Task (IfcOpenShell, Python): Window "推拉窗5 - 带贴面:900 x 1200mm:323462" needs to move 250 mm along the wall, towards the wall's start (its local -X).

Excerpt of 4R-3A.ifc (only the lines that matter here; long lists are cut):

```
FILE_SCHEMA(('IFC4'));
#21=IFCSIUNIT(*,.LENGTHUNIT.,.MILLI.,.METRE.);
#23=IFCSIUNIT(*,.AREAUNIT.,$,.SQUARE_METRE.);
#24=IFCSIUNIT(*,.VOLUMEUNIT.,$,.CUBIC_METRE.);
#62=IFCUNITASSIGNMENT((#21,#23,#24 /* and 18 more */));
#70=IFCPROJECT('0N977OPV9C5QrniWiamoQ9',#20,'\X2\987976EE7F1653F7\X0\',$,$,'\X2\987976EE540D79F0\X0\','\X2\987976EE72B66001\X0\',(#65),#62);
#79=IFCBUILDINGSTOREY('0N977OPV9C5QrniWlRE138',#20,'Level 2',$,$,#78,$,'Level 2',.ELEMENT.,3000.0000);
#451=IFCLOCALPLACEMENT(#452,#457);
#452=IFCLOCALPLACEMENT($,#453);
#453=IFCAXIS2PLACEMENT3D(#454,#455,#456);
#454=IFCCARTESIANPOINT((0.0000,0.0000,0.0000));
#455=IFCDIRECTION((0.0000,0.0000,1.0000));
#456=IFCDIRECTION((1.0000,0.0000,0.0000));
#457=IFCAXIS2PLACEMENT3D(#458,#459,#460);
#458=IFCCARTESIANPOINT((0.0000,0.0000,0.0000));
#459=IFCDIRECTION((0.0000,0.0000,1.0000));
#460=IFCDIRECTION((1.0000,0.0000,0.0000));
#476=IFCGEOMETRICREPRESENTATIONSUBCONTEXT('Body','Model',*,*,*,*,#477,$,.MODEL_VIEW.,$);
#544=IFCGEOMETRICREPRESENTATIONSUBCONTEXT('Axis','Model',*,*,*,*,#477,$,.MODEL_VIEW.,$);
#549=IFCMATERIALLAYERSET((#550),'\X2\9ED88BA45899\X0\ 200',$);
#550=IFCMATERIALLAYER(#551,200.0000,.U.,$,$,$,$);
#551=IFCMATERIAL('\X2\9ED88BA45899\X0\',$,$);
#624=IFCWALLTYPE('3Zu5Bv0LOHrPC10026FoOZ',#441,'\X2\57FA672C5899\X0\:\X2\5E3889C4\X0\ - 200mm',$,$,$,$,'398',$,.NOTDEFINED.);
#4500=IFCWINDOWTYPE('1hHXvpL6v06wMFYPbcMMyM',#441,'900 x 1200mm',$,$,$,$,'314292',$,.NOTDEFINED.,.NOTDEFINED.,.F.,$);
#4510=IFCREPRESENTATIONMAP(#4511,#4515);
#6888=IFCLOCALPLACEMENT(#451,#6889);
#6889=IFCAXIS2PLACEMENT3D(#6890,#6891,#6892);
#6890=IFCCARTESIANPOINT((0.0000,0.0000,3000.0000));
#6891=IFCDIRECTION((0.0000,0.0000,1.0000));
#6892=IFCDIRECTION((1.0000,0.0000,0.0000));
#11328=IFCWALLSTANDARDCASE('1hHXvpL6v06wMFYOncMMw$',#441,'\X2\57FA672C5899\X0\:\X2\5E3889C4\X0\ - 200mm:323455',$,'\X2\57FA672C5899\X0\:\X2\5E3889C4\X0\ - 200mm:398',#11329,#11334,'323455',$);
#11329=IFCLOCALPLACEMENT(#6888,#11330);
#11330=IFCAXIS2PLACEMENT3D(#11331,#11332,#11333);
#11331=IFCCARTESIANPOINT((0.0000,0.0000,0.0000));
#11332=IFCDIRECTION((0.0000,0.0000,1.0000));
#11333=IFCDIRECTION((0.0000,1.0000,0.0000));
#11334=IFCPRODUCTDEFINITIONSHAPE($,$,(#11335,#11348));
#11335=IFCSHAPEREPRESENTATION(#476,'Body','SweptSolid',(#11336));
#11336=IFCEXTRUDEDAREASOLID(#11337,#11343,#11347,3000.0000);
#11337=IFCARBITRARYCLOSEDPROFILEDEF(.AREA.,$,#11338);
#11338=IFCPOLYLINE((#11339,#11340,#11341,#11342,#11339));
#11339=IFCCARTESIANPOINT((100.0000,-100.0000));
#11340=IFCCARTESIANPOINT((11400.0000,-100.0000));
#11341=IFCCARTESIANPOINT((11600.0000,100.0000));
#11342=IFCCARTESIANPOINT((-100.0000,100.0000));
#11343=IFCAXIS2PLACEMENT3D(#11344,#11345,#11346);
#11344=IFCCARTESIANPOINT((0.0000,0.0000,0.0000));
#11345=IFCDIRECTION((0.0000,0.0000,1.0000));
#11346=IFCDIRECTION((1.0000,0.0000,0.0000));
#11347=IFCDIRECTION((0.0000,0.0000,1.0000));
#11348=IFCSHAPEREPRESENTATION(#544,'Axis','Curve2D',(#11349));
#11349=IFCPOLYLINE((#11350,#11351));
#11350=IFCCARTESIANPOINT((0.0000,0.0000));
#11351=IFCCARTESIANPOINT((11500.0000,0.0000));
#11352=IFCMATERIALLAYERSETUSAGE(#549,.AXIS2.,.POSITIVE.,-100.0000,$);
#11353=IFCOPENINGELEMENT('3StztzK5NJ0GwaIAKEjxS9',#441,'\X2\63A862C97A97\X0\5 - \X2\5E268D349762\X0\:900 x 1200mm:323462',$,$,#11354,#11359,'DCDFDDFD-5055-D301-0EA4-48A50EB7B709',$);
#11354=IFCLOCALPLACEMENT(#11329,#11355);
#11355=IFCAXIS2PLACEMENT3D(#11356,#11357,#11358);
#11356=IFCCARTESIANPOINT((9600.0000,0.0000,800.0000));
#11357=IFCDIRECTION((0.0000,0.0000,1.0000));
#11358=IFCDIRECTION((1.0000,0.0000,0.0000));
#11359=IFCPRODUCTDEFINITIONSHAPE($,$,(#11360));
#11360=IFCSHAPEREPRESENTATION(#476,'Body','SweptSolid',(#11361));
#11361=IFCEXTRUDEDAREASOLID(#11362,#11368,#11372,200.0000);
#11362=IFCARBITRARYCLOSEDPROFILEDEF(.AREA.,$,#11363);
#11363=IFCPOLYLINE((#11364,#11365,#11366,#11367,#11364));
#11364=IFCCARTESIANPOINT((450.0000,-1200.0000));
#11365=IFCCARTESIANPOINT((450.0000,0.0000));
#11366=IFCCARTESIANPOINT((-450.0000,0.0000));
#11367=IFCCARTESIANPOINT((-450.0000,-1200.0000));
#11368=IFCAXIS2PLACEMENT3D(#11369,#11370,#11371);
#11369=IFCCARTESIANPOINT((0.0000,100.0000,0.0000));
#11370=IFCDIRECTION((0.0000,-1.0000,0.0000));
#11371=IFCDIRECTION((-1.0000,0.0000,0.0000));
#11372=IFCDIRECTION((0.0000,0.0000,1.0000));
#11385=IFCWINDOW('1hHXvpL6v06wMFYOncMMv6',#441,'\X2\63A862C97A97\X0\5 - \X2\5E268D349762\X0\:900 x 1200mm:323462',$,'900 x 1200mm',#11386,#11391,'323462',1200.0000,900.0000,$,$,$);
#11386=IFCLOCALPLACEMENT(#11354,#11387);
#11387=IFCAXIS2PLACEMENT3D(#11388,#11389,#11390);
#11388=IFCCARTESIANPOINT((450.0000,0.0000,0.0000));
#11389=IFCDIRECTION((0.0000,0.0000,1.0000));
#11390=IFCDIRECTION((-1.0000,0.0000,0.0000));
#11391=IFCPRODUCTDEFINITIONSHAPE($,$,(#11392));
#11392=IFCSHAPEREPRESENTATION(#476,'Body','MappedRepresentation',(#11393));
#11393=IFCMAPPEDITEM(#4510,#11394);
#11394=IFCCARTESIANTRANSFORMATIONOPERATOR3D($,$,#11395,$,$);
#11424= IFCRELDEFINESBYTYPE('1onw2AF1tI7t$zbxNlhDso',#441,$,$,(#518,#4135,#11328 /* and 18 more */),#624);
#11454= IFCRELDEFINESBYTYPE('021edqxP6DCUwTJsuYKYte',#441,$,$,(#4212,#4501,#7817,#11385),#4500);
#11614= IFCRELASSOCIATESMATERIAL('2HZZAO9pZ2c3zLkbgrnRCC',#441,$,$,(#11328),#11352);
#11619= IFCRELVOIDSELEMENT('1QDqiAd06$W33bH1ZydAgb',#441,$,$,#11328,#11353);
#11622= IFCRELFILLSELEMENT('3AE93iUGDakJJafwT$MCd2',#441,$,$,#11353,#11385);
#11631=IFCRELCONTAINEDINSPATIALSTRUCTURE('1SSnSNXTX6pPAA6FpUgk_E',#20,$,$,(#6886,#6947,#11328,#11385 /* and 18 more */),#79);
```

```python
import ifcopenshell
import ifcopenshell.api.geometry
import ifcopenshell.util.placement
import ifcopenshell.util.unit

model = ifcopenshell.open("4R-3A.ifc")
unit_scale = ifcopenshell.util.unit.calculate_unit_scale(model)

window = model.by_guid("1hHXvpL6v06wMFYOncMMv6")
opening = window.FillsVoids[0].RelatingOpeningElement
wall = opening.VoidsElements[0].RelatingBuildingElement

wall_matrix = ifcopenshell.util.placement.get_local_placement(wall.ObjectPlacement)
shift = wall_matrix[:3, 0] * -0.25 / unit_scale
before = ifcopenshell.util.placement.get_local_placement(window.ObjectPlacement)[:3, 3].copy()

# The window is placed relative to its opening, so it follows when the opening moves.
matrix = ifcopenshell.util.placement.get_local_placement(opening.ObjectPlacement)
matrix[:3, 3] += shift
ifcopenshell.api.geometry.edit_object_placement(
    model, product=opening, matrix=matrix, is_si=False, should_transform_children=True
)

after = ifcopenshell.util.placement.get_local_placement(window.ObjectPlacement)[:3, 3]
print("window moved by", (after - before).round(3) + 0.0)

model.write("4R-3A_updated.ifc")
```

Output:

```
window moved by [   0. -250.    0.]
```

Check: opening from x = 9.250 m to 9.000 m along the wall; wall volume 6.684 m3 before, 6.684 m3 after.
